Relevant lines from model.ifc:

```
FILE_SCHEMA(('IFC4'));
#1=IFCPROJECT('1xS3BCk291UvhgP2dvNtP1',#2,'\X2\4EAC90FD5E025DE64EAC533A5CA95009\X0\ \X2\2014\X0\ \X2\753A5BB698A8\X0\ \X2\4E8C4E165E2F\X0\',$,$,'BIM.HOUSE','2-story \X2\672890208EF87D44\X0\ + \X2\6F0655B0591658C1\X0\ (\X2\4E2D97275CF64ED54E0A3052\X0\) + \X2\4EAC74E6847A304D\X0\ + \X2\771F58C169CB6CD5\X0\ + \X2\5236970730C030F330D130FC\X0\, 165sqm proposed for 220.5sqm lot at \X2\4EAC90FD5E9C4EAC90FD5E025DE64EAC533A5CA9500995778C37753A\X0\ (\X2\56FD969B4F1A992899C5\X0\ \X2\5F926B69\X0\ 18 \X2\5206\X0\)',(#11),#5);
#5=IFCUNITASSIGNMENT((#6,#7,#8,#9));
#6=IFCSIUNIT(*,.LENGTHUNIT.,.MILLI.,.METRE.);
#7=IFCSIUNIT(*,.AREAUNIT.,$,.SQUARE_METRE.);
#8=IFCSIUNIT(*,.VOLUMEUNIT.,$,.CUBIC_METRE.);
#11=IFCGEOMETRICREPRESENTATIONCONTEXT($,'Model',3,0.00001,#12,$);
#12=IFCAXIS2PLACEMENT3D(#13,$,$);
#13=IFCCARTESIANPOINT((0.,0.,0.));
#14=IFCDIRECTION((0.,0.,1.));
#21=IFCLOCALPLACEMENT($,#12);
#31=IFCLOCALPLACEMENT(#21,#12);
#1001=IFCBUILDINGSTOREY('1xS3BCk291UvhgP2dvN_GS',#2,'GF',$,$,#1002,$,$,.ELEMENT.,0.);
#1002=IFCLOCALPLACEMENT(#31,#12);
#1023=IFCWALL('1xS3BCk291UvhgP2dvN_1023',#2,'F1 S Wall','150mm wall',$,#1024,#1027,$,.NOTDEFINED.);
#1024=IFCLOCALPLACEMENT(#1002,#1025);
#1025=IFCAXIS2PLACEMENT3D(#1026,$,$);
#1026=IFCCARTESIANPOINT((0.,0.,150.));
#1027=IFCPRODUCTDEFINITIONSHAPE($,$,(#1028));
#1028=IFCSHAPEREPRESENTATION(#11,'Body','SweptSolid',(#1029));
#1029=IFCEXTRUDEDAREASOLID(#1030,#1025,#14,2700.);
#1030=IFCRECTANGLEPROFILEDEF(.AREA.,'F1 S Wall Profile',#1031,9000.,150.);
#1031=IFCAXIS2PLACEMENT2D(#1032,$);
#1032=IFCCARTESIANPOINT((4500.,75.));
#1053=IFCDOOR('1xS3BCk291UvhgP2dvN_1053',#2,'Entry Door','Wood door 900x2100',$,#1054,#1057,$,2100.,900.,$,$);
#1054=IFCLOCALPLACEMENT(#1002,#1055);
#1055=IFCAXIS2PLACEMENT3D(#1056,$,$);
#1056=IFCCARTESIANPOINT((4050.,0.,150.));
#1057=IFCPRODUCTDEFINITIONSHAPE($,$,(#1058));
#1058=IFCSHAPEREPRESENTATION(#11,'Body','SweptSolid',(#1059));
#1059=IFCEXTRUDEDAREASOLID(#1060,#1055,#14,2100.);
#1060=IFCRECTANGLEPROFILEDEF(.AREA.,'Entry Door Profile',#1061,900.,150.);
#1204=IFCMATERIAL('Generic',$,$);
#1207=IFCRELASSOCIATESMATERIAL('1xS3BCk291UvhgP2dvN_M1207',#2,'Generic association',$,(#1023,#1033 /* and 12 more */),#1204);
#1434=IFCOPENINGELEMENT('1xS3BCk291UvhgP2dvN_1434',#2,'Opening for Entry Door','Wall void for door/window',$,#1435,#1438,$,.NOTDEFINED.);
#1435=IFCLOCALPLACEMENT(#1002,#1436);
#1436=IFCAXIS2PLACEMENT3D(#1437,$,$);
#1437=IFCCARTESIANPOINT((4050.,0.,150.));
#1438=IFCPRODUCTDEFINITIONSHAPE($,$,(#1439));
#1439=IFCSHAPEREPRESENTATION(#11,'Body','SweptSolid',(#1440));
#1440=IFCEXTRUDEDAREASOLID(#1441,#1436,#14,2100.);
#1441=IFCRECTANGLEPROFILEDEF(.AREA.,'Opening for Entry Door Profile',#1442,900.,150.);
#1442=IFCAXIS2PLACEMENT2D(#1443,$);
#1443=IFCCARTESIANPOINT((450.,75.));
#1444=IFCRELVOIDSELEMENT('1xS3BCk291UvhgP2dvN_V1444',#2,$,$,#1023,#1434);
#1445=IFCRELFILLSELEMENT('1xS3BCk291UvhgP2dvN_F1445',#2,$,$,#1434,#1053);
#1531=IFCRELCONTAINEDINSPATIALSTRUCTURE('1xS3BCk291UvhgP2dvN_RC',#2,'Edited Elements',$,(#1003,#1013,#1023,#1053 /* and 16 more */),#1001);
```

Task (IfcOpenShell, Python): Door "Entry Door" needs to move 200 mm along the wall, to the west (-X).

```python
import ifcopenshell
import ifcopenshell.api.geometry
import ifcopenshell.util.placement

model = ifcopenshell.open("model.ifc")

door = model.by_id(1053)
opening = door.FillsVoids[0].RelatingOpeningElement
wall = opening.VoidsElements[0].RelatingBuildingElement

wall_matrix = ifcopenshell.util.placement.get_local_placement(wall.ObjectPlacement)
shift = wall_matrix[:3, 0] * -200.0
before = ifcopenshell.util.placement.get_local_placement(door.ObjectPlacement)[:3, 3].copy()

# The door is not placed relative to its opening, so move both.
for product in (opening, door):
    matrix = ifcopenshell.util.placement.get_local_placement(product.ObjectPlacement)
    matrix[:3, 3] += shift
    ifcopenshell.api.geometry.edit_object_placement(model, product=product, matrix=matrix, is_si=False)

after = ifcopenshell.util.placement.get_local_placement(door.ObjectPlacement)[:3, 3]
print("door moved by", (after - before).round(3) + 0.0)

model.write("model_edited.ifc")
```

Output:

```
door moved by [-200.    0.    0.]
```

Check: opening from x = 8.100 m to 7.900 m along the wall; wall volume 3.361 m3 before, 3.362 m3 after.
